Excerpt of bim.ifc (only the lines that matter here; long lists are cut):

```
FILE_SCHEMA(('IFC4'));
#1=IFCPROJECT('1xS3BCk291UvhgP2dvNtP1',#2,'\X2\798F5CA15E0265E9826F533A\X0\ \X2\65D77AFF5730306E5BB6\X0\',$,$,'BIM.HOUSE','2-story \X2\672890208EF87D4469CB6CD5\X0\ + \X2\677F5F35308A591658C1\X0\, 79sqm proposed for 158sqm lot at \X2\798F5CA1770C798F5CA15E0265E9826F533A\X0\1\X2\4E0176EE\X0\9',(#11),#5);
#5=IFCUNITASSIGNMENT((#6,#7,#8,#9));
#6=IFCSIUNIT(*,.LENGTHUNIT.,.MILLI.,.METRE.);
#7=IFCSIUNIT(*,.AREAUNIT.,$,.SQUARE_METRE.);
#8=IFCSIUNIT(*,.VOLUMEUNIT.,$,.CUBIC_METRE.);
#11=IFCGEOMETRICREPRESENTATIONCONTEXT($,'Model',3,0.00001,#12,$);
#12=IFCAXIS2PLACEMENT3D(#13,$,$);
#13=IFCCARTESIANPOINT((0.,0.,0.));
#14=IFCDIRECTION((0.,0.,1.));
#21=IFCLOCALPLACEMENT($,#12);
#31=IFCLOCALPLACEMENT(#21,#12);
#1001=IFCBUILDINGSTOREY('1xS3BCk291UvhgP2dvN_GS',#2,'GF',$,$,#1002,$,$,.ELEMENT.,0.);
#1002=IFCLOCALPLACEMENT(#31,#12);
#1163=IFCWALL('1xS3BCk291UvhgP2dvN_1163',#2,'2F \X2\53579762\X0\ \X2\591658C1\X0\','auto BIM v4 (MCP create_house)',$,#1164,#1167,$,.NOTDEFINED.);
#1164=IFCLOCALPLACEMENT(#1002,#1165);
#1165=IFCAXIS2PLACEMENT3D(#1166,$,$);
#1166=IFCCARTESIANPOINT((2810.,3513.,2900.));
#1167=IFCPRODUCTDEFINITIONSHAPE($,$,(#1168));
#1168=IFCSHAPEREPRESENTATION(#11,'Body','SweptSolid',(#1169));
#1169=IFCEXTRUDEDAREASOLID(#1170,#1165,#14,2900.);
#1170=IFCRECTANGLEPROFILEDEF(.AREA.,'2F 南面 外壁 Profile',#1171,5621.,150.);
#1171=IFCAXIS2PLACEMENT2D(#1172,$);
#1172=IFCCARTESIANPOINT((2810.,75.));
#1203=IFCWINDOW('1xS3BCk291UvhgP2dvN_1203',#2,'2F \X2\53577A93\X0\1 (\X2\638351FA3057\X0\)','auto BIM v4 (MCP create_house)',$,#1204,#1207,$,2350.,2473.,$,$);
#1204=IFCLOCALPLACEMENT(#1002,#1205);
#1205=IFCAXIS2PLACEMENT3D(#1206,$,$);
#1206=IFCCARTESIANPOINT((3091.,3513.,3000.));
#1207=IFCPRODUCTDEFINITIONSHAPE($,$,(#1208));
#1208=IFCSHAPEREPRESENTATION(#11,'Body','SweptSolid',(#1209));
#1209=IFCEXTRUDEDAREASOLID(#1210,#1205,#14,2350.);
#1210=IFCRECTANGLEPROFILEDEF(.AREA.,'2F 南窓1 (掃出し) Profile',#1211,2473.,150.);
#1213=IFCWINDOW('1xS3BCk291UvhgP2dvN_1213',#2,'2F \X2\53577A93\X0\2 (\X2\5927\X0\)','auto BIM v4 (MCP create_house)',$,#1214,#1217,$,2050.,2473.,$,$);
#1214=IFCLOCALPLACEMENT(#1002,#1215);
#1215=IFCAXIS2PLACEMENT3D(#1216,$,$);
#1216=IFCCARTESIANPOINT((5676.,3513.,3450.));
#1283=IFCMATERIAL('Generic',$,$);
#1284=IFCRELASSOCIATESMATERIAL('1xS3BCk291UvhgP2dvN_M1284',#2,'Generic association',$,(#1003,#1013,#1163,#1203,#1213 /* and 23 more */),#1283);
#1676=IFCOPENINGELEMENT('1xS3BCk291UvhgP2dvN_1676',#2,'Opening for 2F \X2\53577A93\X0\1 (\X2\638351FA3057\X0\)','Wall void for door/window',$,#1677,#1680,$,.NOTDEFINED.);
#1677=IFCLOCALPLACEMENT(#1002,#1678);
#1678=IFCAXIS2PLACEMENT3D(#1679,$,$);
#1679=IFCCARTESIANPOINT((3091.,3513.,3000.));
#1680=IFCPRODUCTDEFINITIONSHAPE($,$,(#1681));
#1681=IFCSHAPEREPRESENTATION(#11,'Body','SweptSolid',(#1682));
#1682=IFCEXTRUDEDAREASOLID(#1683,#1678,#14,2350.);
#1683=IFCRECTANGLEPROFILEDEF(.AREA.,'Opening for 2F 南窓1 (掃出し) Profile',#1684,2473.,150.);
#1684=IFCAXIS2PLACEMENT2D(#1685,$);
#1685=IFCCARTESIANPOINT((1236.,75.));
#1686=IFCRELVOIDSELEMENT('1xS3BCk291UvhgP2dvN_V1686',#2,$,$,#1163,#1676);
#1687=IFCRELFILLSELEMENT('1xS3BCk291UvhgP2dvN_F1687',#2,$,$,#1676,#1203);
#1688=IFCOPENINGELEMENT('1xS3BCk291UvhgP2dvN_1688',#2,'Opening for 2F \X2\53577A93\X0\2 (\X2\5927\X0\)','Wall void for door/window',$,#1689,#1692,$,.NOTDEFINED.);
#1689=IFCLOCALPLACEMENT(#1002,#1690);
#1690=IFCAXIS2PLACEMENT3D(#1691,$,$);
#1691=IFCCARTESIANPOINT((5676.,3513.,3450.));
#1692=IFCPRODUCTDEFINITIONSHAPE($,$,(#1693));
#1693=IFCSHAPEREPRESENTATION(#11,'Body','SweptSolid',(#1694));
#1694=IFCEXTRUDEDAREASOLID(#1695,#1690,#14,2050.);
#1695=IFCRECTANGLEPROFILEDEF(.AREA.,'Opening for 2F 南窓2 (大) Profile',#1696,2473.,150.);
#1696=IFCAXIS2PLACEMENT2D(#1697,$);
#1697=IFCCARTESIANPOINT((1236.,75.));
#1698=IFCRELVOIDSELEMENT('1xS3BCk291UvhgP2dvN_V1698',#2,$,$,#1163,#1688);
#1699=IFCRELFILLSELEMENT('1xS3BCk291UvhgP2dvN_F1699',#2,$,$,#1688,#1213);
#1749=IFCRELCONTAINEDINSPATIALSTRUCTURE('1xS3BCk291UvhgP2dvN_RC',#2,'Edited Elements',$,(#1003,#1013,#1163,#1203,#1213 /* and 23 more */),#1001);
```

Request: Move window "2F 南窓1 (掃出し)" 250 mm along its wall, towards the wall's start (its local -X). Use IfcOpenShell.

```python
import ifcopenshell
import ifcopenshell.api.geometry
import ifcopenshell.util.placement

model = ifcopenshell.open("bim.ifc")

window = model.by_guid("1xS3BCk291UvhgP2dvN_1203")
opening = window.FillsVoids[0].RelatingOpeningElement
wall = opening.VoidsElements[0].RelatingBuildingElement

wall_matrix = ifcopenshell.util.placement.get_local_placement(wall.ObjectPlacement)
shift = wall_matrix[:3, 0] * -250.0
before = ifcopenshell.util.placement.get_local_placement(window.ObjectPlacement)[:3, 3].copy()

# The window is not placed relative to its opening, so move both.
for product in (opening, window):
    matrix = ifcopenshell.util.placement.get_local_placement(product.ObjectPlacement)
    matrix[:3, 3] += shift
    ifcopenshell.api.geometry.edit_object_placement(model, product=product, matrix=matrix, is_si=False)

after = ifcopenshell.util.placement.get_local_placement(window.ObjectPlacement)[:3, 3]
print("window moved by", (after - before).round(3) + 0.0)

model.write("bim_v2.ifc")
```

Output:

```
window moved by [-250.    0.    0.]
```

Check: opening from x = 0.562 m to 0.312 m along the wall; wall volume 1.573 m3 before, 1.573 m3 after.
